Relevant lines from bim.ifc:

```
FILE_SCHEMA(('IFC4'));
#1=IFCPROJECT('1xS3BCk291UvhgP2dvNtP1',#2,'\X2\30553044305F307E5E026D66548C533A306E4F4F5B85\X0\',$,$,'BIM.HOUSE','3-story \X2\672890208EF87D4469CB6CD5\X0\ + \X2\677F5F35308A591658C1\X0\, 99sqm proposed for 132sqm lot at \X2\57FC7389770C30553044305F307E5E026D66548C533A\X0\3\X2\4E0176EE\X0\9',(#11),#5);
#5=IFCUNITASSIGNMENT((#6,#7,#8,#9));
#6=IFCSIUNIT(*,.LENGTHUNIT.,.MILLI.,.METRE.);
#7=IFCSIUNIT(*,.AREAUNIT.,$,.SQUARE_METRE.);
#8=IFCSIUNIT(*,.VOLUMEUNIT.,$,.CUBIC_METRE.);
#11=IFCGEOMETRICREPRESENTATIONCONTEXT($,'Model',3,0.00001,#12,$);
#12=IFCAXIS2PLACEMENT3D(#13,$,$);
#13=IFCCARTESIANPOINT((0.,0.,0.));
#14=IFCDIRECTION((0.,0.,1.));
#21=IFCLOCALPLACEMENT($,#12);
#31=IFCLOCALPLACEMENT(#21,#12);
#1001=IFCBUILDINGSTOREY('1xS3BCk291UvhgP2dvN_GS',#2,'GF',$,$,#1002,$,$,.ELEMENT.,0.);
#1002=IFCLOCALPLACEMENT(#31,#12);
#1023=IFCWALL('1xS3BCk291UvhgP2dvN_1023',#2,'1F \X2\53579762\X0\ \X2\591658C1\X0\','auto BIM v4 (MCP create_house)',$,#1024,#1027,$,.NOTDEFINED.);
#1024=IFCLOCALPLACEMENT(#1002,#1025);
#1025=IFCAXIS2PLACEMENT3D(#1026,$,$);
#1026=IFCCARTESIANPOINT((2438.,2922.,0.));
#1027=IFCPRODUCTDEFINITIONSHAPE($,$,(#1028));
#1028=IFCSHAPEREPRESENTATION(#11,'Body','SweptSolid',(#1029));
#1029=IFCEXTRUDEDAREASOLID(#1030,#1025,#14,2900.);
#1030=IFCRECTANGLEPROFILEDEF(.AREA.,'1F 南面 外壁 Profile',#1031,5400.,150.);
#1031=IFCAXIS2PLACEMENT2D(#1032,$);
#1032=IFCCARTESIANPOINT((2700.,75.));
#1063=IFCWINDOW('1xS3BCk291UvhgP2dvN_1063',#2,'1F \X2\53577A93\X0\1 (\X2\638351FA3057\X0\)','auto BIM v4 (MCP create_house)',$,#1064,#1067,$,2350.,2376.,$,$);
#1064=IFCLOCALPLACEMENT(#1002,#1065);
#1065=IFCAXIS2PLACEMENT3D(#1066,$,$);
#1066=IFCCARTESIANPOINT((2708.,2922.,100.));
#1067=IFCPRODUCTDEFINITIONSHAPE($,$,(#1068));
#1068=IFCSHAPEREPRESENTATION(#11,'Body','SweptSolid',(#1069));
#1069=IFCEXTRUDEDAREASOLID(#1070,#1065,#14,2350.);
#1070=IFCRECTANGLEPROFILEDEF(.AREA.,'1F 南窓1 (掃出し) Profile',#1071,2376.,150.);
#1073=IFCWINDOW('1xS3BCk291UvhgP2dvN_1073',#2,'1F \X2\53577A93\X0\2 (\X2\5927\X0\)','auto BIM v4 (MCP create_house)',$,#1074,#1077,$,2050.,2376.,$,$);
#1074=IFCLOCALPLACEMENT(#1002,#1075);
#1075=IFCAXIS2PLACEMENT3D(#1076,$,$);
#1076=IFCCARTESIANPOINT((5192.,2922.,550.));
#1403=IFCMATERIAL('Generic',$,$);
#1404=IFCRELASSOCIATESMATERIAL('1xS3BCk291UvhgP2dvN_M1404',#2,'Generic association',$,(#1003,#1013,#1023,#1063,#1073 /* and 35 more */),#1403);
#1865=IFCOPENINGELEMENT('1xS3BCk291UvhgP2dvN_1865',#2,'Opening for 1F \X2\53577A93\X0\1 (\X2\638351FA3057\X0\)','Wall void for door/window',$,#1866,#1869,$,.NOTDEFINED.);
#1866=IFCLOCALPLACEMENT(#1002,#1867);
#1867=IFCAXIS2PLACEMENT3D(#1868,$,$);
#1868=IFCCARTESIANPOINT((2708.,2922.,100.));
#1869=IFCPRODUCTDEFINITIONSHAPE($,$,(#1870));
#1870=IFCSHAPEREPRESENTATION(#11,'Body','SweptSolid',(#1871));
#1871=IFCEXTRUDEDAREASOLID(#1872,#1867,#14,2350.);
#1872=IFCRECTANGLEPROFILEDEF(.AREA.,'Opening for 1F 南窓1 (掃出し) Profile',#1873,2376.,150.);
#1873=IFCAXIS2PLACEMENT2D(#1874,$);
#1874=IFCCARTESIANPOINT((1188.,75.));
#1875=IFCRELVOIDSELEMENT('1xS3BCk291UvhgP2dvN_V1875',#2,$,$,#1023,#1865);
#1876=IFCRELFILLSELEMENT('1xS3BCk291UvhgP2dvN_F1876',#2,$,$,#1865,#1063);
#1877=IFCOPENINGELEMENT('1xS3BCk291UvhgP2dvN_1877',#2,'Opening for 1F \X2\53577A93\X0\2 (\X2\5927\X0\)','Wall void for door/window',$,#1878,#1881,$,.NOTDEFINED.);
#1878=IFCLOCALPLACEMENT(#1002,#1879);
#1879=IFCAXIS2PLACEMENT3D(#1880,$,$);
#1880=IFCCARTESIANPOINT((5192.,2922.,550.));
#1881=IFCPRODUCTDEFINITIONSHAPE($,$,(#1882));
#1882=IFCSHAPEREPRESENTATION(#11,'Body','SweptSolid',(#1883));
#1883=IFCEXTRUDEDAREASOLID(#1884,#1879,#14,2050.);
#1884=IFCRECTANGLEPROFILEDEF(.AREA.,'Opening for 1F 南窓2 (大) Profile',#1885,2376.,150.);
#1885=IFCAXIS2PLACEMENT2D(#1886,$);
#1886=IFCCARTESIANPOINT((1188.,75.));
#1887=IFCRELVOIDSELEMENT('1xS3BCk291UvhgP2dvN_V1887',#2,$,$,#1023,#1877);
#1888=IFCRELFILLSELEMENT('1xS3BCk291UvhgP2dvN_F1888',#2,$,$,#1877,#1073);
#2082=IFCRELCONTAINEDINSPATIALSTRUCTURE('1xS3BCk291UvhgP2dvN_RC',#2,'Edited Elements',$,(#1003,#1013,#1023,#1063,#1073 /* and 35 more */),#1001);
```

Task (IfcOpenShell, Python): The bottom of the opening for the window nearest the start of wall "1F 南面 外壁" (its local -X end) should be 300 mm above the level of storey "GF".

```python
import numpy as np
import ifcopenshell
import ifcopenshell.api.geometry
import ifcopenshell.geom
import ifcopenshell.util.element
import ifcopenshell.util.placement
import ifcopenshell.util.shape
import ifcopenshell.util.unit

model = ifcopenshell.open("bim.ifc")
unit_scale = ifcopenshell.util.unit.calculate_unit_scale(model)

window = model.by_guid("1xS3BCk291UvhgP2dvN_1063")
opening = window.FillsVoids[0].RelatingOpeningElement
storey = ifcopenshell.util.element.get_container(window, ifc_class="IfcBuildingStorey")
level = ifcopenshell.util.placement.get_local_placement(storey.ObjectPlacement)[2, 3]

# The opening's origin need not be at the sill, so measure its lowest point.
shape = ifcopenshell.geom.create_shape(ifcopenshell.geom.settings(), opening)
bottom = ifcopenshell.util.shape.get_shape_bottom_elevation(shape, shape.geometry) / unit_scale
dz = level + 0.3 / unit_scale - bottom

shift = np.array([0.0, 0.0, dz])
# The window is not placed relative to its opening, so move both.
for product in (opening, window):
    matrix = ifcopenshell.util.placement.get_local_placement(product.ObjectPlacement)
    matrix[:3, 3] += shift
    ifcopenshell.api.geometry.edit_object_placement(model, product=product, matrix=matrix, is_si=False)

print(f"moved by {dz * unit_scale:+.3f} m")

model.write("bim_rev.ifc")
```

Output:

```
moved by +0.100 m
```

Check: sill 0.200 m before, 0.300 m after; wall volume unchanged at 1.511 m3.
